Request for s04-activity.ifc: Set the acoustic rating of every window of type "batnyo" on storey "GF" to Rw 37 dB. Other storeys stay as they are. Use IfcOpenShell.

First a look at what the model holds.

```python
import ifcopenshell
import ifcopenshell.util.element

model = ifcopenshell.open("s04-activity.ifc")
print(model.schema)
storey = next(s for s in model.by_type("IfcBuildingStorey") if s.Name == "GF")
windows = [e for e in ifcopenshell.util.element.get_decomposition(storey) if e.is_a("IfcWindow")]
seen = {}
for e in windows:
    element_type = ifcopenshell.util.element.get_type(e)
    key = (element_type.Name if element_type != e and element_type else None, ifcopenshell.util.element.get_pset(e, "Pset_WindowCommon", "AcousticRating"))
    seen[key] = seen.get(key, 0) + 1
for (name, value), count in sorted(seen.items(), key=str):
    print(count, "x", name, "|", value)
```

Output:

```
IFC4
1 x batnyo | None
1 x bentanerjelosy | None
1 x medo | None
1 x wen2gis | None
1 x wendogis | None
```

```python
import ifcopenshell
import ifcopenshell.api.pset
import ifcopenshell.util.element

model = ifcopenshell.open("s04-activity.ifc")

storey = next(s for s in model.by_type("IfcBuildingStorey") if s.Name == "GF")
windows = [e for e in ifcopenshell.util.element.get_decomposition(storey) if e.is_a("IfcWindow")]

count = 0
for e in windows:
    element_type = ifcopenshell.util.element.get_type(e)
    if element_type in (None, e) or element_type.Name != "batnyo":
        continue
    # add_pset returns the element's existing set when there is one.
    pset = ifcopenshell.api.pset.add_pset(model, product=e, name="Pset_WindowCommon")
    ifcopenshell.api.pset.edit_pset(model, pset=pset, properties={"AcousticRating": "Rw 37 dB"})
    count += 1

print(count, "windows updated")

model.write("s04-activity_updated.ifc")
```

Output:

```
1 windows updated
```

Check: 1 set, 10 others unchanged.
